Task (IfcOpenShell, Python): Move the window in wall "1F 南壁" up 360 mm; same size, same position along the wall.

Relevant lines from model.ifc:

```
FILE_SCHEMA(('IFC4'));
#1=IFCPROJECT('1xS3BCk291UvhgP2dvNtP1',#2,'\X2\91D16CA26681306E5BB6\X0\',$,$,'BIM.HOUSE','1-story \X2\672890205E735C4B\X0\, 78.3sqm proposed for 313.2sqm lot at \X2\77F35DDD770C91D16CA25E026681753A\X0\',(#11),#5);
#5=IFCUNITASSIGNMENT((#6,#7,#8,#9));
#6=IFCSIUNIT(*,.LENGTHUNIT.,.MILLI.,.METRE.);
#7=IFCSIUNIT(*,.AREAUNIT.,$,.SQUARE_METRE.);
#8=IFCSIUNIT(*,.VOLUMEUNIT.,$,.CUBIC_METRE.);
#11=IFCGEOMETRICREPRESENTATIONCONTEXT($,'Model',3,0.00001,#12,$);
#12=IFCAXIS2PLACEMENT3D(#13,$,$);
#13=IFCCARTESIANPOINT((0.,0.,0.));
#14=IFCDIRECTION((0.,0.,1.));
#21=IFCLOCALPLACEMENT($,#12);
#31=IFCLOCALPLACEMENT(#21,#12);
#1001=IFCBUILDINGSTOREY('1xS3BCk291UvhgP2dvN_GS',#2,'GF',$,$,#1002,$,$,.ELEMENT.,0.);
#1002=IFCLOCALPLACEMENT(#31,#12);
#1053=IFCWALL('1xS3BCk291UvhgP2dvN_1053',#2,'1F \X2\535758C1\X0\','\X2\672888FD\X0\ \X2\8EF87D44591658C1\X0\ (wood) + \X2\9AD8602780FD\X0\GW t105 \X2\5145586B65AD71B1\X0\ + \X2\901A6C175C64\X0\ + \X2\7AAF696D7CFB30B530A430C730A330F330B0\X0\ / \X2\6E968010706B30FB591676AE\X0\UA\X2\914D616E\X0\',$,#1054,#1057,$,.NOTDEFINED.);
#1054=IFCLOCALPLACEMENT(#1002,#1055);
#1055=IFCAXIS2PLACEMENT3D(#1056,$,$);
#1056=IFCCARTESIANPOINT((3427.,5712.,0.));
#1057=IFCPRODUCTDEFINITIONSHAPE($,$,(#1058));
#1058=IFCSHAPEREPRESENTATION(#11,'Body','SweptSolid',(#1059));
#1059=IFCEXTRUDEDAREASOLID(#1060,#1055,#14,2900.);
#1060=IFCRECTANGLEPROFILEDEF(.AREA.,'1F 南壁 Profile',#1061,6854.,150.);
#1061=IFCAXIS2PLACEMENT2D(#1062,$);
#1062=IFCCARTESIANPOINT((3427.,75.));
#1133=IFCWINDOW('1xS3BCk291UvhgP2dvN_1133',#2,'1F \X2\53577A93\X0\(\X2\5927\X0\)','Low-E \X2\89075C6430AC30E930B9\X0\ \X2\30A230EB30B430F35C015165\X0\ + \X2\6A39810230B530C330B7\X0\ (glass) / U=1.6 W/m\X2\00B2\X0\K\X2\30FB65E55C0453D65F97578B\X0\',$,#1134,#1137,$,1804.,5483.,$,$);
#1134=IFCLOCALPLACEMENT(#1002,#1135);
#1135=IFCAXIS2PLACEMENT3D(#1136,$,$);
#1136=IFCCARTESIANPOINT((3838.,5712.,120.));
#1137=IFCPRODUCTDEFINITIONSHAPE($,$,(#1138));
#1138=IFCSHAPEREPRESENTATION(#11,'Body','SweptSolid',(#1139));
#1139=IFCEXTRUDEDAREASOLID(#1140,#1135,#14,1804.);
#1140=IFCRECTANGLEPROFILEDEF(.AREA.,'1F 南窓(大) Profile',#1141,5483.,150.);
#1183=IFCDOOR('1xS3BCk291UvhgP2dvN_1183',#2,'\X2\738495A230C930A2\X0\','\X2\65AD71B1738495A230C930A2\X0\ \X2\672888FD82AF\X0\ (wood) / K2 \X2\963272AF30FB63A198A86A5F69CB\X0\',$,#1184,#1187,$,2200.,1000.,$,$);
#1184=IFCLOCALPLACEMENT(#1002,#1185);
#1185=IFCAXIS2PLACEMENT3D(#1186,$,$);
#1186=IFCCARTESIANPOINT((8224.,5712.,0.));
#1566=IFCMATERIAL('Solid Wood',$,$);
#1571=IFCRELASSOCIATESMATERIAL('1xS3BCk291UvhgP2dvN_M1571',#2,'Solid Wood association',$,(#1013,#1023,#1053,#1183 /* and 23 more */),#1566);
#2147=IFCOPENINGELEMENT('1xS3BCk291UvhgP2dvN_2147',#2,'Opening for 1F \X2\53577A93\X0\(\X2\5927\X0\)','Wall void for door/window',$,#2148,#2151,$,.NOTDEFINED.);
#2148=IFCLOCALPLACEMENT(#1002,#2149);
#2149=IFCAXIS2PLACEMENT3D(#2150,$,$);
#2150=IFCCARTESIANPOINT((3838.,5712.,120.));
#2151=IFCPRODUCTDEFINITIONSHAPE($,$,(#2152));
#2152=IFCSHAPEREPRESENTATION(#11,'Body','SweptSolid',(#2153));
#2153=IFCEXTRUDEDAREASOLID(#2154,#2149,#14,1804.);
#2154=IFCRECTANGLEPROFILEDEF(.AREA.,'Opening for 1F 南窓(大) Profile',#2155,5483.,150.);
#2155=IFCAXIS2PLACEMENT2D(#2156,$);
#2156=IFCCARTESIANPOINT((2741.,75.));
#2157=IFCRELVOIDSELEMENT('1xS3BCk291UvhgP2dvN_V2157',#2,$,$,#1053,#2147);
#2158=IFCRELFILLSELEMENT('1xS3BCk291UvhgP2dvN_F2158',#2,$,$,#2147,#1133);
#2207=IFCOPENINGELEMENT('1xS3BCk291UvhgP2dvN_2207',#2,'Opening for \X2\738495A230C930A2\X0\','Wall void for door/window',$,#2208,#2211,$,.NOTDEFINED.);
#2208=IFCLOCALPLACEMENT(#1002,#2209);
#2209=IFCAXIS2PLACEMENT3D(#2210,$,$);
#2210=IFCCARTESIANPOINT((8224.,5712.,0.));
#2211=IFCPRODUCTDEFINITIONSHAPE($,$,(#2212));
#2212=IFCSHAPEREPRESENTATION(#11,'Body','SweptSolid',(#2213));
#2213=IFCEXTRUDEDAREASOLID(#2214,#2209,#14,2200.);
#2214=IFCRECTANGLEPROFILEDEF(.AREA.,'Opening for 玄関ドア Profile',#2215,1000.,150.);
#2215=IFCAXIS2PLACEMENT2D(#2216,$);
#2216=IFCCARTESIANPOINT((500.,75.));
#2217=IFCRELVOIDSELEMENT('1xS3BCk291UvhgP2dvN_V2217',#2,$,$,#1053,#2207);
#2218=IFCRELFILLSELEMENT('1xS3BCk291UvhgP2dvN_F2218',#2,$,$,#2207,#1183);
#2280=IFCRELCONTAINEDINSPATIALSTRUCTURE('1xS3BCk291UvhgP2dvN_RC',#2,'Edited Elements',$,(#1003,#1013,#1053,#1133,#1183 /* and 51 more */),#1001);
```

```python
import numpy as np
import ifcopenshell
import ifcopenshell.api.geometry
import ifcopenshell.util.placement
import ifcopenshell.util.unit

model = ifcopenshell.open("model.ifc")
unit_scale = ifcopenshell.util.unit.calculate_unit_scale(model)

window = model.by_guid("1xS3BCk291UvhgP2dvN_1133")
opening = window.FillsVoids[0].RelatingOpeningElement
dz = 360.0

shift = np.array([0.0, 0.0, dz])
# The window is not placed relative to its opening, so move both.
for product in (opening, window):
    matrix = ifcopenshell.util.placement.get_local_placement(product.ObjectPlacement)
    matrix[:3, 3] += shift
    ifcopenshell.api.geometry.edit_object_placement(model, product=product, matrix=matrix, is_si=False)

print(f"moved by {dz * unit_scale:+.3f} m")

model.write("model_rev.ifc")
```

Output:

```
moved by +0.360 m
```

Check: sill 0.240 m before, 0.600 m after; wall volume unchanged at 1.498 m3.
